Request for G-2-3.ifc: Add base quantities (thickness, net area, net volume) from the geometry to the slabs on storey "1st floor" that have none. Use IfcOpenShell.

First a look at what the model holds.

```python
import ifcopenshell
import ifcopenshell.util.element
import ifcopenshell.util.unit

model = ifcopenshell.open("G-2-3.ifc")
print(model.schema)
for unit_type in ("LENGTHUNIT", "AREAUNIT", "VOLUMEUNIT"):
    print(unit_type, ifcopenshell.util.unit.calculate_unit_scale(model, unit_type))
storey = next(s for s in model.by_type("IfcBuildingStorey") if s.Name == "1st floor")
slabs = [e for e in ifcopenshell.util.element.get_decomposition(storey) if e.is_a("IfcSlab")]
for e in sorted(slabs, key=lambda e: e.id()):
    print(e.id(), e.is_a(), e.Name, list(ifcopenshell.util.element.get_psets(e, qtos_only=True)), sep=" | ")
```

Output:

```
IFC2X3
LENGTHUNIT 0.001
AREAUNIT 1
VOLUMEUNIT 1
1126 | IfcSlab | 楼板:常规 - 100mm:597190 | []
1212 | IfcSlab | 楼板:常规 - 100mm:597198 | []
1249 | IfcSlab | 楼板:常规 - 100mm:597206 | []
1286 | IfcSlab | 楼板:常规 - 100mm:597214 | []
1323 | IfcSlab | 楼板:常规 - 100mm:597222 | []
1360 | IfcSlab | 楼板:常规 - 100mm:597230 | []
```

```python
import ifcopenshell
import ifcopenshell.api.pset
import ifcopenshell.geom
import ifcopenshell.util.element
import ifcopenshell.util.shape
import ifcopenshell.util.unit

model = ifcopenshell.open("G-2-3.ifc")
unit_scale = ifcopenshell.util.unit.calculate_unit_scale(model)
area_scale = ifcopenshell.util.unit.calculate_unit_scale(model, "AREAUNIT")
volume_scale = ifcopenshell.util.unit.calculate_unit_scale(model, "VOLUMEUNIT")
settings = ifcopenshell.geom.settings()

storey = next(s for s in model.by_type("IfcBuildingStorey") if s.Name == "1st floor")
slabs = [e for e in ifcopenshell.util.element.get_decomposition(storey) if e.is_a("IfcSlab")]

for e in sorted(slabs, key=lambda e: e.id()):
    if ifcopenshell.util.element.get_psets(e, qtos_only=True, should_inherit=False):
        continue
    # Geometry comes back in metres, in the element's own axes.
    shape = ifcopenshell.geom.create_shape(settings, e)
    values = {
        "Width": ifcopenshell.util.shape.get_z(shape.geometry) / unit_scale,
        "NetArea": ifcopenshell.util.shape.get_footprint_area(shape.geometry) / area_scale,
        "NetVolume": ifcopenshell.util.shape.get_volume(shape.geometry) / volume_scale,
    }
    qto = ifcopenshell.api.pset.add_qto(model, product=e, name="BaseQuantities")
    ifcopenshell.api.pset.edit_qto(model, qto=qto, properties=values)
    print(e.id(), {k: round(v, 3) for k, v in values.items()})

model.write("G-2-3_edited.ifc")
```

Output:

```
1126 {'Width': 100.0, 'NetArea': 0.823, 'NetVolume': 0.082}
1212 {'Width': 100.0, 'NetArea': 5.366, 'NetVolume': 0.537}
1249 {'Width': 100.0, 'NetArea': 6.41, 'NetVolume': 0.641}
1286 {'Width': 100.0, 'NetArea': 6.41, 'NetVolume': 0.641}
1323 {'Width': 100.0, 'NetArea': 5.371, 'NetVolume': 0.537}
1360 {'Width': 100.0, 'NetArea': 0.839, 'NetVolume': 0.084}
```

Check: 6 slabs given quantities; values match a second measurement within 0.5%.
